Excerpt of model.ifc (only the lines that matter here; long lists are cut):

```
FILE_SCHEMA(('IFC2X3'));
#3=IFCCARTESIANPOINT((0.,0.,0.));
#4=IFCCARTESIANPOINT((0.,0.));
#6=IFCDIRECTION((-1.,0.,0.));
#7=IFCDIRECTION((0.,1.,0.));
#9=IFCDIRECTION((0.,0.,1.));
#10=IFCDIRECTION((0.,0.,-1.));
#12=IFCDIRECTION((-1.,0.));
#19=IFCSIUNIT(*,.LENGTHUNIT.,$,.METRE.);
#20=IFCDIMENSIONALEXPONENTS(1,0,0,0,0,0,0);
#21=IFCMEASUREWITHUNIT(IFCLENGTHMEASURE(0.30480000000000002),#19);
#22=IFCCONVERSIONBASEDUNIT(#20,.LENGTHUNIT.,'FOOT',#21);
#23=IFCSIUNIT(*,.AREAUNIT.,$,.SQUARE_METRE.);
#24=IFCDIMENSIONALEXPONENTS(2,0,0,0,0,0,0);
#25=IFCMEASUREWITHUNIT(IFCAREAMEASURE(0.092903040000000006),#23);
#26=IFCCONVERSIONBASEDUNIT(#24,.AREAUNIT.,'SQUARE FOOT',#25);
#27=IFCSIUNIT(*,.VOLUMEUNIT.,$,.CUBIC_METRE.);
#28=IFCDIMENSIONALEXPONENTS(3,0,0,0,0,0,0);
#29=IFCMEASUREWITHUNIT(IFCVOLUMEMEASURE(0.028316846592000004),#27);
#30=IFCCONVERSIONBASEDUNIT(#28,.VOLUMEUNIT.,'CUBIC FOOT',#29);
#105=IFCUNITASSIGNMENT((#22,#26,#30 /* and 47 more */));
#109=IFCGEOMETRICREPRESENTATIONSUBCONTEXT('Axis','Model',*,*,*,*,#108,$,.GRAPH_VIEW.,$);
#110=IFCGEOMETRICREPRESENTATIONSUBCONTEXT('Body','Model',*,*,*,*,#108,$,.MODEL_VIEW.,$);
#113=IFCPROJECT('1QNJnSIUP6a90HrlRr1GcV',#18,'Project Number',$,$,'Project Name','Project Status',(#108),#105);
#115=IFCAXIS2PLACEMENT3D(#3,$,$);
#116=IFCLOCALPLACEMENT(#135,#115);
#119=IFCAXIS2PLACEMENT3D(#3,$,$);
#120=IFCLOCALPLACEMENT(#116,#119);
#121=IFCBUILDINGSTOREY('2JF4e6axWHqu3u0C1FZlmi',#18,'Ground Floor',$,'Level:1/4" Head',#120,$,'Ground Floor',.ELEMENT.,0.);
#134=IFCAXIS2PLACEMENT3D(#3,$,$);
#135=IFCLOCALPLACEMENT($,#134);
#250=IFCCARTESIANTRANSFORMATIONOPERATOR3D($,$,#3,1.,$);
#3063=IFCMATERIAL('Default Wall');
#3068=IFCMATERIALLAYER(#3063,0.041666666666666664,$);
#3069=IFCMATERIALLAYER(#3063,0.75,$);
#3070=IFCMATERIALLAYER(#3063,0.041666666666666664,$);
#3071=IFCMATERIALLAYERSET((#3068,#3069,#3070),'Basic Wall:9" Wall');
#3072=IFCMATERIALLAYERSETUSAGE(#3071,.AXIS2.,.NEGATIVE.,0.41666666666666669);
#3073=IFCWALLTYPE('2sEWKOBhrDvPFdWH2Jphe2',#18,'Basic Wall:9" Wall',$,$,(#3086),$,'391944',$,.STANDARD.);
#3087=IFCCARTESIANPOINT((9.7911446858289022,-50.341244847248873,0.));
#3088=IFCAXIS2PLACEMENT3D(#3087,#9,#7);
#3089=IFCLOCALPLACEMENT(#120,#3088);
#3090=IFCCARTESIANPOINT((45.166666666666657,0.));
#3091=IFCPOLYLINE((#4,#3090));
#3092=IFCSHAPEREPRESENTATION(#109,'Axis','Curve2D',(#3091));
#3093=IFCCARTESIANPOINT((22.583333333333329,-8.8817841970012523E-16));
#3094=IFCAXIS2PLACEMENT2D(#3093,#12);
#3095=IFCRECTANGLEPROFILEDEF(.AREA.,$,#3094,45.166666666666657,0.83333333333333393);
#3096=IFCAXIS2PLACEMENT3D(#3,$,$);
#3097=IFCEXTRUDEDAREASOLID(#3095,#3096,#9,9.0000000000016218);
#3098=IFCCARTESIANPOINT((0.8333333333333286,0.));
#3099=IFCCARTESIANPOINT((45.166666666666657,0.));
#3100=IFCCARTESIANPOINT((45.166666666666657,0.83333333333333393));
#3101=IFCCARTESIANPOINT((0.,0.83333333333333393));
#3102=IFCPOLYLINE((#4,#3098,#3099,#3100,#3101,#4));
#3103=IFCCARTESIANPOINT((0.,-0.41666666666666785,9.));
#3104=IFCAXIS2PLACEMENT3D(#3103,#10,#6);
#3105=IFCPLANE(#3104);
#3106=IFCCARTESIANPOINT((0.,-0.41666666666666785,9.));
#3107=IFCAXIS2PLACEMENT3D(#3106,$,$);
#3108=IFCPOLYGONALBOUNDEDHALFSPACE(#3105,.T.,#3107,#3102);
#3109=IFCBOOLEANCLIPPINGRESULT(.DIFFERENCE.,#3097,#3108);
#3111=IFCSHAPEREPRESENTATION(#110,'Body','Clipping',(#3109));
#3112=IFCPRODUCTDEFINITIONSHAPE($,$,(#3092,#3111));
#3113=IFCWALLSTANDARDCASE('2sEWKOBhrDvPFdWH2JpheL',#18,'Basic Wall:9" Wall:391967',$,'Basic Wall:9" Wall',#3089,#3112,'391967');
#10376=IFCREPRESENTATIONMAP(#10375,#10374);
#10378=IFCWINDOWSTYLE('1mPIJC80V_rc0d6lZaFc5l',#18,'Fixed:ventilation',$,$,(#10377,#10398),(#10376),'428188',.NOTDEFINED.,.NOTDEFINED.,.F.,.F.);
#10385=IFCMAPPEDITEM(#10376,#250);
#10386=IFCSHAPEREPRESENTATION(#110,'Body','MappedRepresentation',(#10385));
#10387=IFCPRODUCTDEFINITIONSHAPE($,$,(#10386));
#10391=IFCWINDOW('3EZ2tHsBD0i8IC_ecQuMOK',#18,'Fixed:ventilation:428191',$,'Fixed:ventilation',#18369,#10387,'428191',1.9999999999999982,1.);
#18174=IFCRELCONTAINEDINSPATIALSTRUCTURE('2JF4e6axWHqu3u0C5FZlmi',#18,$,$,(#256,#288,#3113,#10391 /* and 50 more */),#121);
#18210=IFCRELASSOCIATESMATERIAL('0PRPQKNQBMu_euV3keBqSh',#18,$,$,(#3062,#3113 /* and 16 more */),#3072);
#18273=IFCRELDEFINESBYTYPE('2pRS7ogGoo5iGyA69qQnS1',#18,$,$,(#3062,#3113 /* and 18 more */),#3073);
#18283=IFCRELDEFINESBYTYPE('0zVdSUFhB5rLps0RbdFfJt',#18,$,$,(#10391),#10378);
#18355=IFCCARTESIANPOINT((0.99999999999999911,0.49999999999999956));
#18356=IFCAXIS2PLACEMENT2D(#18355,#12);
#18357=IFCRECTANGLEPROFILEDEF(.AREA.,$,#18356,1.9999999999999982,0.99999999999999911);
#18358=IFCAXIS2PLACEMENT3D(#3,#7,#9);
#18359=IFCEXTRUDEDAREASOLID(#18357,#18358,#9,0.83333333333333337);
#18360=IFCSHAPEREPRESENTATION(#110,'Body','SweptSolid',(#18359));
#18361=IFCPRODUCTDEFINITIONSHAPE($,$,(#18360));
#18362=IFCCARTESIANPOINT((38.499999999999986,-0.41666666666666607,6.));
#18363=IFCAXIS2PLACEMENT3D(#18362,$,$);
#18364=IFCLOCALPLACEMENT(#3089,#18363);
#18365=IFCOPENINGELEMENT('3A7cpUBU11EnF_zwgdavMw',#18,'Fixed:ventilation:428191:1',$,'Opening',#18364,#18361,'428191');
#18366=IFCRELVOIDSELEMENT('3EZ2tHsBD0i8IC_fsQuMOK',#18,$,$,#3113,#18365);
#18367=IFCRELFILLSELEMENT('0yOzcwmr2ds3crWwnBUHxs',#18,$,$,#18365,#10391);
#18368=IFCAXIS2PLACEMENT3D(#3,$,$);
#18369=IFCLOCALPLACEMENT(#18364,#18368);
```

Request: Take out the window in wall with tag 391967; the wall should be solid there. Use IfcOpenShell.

```python
import ifcopenshell
import ifcopenshell.api.feature
import ifcopenshell.api.root
import ifcopenshell.geom
import ifcopenshell.util.shape

model = ifcopenshell.open("model.ifc")
settings = ifcopenshell.geom.settings()


def volume(element):
    """Net volume in cubic metres, openings subtracted."""
    shape = ifcopenshell.geom.create_shape(settings, element)
    return ifcopenshell.util.shape.get_volume(shape.geometry)


window = model.by_id(10391)
opening = window.FillsVoids[0].RelatingOpeningElement
wall = opening.VoidsElements[0].RelatingBuildingElement
before = volume(wall)

ifcopenshell.api.root.remove_product(model, product=window)
ifcopenshell.api.feature.remove_feature(model, feature=opening)

after = volume(wall)

print(f"wall volume {before:.3f} -> {after:.3f} m3")

model.write("model_rev.ifc")
```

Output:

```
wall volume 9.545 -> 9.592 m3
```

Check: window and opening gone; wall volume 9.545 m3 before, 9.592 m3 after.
